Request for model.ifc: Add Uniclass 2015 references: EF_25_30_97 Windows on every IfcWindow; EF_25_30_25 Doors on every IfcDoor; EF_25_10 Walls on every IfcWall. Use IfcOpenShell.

First a look at what the model holds.

```python
import ifcopenshell

model = ifcopenshell.open("model.ifc")
print(model.schema)
print("classifications:", [c.Name for c in model.by_type("IfcClassification")])
for ifc_class in ("IfcDoor", "IfcRoof", "IfcStair", "IfcWall", "IfcWindow"):
    print(ifc_class, len(model.by_type(ifc_class)))
```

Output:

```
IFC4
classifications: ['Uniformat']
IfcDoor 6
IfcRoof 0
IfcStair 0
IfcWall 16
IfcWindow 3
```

```python
import ifcopenshell
import ifcopenshell.api.classification

model = ifcopenshell.open("model.ifc")

system = ifcopenshell.api.classification.add_classification(model, classification="Uniclass 2015")

codes = {
    "IfcWindow": ("EF_25_30_97", "Windows"),
    "IfcDoor": ("EF_25_30_25", "Doors"),
    "IfcWall": ("EF_25_10", "Walls"),
}
for ifc_class, (code, name) in codes.items():
    products = model.by_type(ifc_class)
    ifcopenshell.api.classification.add_reference(
        model, products=products, classification=system, identification=code, name=name
    )
    print(code, len(products))

model.write("model_edited.ifc")
```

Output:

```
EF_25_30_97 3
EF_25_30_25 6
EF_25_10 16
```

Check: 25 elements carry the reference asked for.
